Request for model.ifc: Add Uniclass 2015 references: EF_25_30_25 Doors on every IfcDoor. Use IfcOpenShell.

First a look at what the model holds.

```python
import ifcopenshell

model = ifcopenshell.open("model.ifc")
print(model.schema)
print("classifications:", [c.Name for c in model.by_type("IfcClassification")])
for ifc_class in ("IfcDoor", "IfcRoof", "IfcStair", "IfcWall", "IfcWindow"):
    print(ifc_class, len(model.by_type(ifc_class)))
```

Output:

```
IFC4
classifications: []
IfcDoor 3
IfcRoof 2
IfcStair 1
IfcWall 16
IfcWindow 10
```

```python
import ifcopenshell
import ifcopenshell.api.classification

model = ifcopenshell.open("model.ifc")

system = ifcopenshell.api.classification.add_classification(model, classification="Uniclass 2015")

codes = {
    "IfcDoor": ("EF_25_30_25", "Doors"),
}
for ifc_class, (code, name) in codes.items():
    products = model.by_type(ifc_class)
    ifcopenshell.api.classification.add_reference(
        model, products=products, classification=system, identification=code, name=name
    )
    print(code, len(products))

model.write("model-out.ifc")
```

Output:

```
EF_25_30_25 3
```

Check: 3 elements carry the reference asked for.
